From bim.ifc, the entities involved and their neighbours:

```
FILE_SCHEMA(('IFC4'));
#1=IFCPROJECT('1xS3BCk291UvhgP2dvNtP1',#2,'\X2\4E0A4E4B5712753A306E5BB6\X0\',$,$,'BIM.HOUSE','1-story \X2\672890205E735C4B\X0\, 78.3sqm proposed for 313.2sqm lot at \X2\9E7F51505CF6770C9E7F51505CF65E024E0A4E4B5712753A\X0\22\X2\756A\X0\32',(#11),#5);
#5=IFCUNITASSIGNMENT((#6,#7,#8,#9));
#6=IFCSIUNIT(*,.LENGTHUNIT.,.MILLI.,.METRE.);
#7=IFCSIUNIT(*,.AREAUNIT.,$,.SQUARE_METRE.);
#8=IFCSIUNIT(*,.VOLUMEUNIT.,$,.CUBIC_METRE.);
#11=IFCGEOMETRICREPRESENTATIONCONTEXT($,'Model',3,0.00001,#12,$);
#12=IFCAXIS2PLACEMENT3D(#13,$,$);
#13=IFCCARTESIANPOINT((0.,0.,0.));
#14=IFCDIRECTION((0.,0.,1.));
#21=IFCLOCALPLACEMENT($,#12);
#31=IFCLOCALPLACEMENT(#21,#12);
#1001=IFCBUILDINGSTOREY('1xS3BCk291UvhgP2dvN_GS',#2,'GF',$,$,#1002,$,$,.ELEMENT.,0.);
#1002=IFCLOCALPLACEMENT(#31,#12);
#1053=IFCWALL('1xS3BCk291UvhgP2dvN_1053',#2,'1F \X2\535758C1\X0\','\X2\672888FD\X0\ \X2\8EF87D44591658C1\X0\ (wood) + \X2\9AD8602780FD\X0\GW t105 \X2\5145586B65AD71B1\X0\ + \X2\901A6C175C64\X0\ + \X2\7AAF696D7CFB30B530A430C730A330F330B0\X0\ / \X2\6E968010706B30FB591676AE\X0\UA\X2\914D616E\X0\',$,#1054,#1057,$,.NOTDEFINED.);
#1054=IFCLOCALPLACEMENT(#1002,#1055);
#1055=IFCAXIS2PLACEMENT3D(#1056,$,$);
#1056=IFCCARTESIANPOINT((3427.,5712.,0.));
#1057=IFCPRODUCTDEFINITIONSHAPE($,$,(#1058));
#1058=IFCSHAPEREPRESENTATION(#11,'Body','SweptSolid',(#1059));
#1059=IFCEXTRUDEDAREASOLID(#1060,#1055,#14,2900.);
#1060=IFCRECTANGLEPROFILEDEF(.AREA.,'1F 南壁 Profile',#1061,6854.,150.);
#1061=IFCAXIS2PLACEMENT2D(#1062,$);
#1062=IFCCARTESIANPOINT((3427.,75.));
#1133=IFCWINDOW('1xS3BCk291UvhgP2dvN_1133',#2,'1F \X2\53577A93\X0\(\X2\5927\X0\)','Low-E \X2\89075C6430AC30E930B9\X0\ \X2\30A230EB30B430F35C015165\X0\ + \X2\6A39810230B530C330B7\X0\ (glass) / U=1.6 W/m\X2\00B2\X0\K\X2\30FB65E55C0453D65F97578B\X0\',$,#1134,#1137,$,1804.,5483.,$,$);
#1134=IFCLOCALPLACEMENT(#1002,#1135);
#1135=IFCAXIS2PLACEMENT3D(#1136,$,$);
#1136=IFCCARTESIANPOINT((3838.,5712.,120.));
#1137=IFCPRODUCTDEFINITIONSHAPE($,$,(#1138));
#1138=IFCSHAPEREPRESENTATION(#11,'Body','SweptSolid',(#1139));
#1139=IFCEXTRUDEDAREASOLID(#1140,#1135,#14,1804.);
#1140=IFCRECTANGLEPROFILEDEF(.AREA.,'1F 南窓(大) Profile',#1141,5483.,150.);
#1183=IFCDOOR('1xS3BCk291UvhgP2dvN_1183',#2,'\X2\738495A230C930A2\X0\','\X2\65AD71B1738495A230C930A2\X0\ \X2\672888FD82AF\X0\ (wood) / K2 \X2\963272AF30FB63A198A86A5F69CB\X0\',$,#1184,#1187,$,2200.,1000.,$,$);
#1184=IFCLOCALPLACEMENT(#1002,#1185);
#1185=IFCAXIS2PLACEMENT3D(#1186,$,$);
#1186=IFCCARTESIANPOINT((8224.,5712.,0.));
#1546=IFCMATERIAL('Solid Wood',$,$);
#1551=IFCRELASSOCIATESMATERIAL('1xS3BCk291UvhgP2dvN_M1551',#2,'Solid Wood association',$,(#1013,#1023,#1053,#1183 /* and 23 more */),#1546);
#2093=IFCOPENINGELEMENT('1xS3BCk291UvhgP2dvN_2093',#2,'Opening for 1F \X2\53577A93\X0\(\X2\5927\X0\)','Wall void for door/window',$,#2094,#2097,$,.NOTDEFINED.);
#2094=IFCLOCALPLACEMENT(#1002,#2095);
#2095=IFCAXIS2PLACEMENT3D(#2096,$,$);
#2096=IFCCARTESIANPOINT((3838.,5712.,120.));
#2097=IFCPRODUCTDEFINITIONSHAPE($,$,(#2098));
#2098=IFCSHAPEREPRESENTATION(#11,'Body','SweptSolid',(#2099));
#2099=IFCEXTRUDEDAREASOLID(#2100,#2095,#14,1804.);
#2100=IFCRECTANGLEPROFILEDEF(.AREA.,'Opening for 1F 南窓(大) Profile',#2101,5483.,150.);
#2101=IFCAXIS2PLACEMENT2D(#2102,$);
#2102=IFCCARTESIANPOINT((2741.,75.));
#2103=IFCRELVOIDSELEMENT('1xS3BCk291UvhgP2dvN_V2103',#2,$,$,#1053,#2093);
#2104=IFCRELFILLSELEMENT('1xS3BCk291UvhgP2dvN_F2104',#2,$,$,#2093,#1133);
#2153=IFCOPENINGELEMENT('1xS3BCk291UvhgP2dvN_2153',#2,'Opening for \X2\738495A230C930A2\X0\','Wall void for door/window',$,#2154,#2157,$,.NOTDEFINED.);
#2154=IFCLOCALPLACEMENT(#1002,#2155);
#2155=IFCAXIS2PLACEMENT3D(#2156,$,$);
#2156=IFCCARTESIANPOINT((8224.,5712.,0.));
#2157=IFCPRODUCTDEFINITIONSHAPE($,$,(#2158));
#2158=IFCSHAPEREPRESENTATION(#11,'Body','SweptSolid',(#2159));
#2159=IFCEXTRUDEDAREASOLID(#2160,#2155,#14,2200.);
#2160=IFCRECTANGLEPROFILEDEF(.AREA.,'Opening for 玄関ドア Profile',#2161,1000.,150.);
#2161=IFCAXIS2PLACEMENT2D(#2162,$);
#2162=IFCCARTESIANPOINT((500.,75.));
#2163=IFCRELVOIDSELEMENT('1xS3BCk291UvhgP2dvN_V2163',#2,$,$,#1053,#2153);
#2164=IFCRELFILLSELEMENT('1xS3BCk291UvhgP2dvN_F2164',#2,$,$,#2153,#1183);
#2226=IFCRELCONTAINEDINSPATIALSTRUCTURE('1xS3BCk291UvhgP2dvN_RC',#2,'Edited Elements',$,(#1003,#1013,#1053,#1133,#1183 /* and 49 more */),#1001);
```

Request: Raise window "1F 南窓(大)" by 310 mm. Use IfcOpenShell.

```python
import numpy as np
import ifcopenshell
import ifcopenshell.api.geometry
import ifcopenshell.util.placement
import ifcopenshell.util.unit

model = ifcopenshell.open("bim.ifc")
unit_scale = ifcopenshell.util.unit.calculate_unit_scale(model)

window = model.by_guid("1xS3BCk291UvhgP2dvN_1133")
opening = window.FillsVoids[0].RelatingOpeningElement
dz = 310.0

shift = np.array([0.0, 0.0, dz])
# The window is not placed relative to its opening, so move both.
for product in (opening, window):
    matrix = ifcopenshell.util.placement.get_local_placement(product.ObjectPlacement)
    matrix[:3, 3] += shift
    ifcopenshell.api.geometry.edit_object_placement(model, product=product, matrix=matrix, is_si=False)

print(f"moved by {dz * unit_scale:+.3f} m")

model.write("bim-out.ifc")
```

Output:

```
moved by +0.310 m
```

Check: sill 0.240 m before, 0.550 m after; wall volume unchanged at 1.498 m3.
